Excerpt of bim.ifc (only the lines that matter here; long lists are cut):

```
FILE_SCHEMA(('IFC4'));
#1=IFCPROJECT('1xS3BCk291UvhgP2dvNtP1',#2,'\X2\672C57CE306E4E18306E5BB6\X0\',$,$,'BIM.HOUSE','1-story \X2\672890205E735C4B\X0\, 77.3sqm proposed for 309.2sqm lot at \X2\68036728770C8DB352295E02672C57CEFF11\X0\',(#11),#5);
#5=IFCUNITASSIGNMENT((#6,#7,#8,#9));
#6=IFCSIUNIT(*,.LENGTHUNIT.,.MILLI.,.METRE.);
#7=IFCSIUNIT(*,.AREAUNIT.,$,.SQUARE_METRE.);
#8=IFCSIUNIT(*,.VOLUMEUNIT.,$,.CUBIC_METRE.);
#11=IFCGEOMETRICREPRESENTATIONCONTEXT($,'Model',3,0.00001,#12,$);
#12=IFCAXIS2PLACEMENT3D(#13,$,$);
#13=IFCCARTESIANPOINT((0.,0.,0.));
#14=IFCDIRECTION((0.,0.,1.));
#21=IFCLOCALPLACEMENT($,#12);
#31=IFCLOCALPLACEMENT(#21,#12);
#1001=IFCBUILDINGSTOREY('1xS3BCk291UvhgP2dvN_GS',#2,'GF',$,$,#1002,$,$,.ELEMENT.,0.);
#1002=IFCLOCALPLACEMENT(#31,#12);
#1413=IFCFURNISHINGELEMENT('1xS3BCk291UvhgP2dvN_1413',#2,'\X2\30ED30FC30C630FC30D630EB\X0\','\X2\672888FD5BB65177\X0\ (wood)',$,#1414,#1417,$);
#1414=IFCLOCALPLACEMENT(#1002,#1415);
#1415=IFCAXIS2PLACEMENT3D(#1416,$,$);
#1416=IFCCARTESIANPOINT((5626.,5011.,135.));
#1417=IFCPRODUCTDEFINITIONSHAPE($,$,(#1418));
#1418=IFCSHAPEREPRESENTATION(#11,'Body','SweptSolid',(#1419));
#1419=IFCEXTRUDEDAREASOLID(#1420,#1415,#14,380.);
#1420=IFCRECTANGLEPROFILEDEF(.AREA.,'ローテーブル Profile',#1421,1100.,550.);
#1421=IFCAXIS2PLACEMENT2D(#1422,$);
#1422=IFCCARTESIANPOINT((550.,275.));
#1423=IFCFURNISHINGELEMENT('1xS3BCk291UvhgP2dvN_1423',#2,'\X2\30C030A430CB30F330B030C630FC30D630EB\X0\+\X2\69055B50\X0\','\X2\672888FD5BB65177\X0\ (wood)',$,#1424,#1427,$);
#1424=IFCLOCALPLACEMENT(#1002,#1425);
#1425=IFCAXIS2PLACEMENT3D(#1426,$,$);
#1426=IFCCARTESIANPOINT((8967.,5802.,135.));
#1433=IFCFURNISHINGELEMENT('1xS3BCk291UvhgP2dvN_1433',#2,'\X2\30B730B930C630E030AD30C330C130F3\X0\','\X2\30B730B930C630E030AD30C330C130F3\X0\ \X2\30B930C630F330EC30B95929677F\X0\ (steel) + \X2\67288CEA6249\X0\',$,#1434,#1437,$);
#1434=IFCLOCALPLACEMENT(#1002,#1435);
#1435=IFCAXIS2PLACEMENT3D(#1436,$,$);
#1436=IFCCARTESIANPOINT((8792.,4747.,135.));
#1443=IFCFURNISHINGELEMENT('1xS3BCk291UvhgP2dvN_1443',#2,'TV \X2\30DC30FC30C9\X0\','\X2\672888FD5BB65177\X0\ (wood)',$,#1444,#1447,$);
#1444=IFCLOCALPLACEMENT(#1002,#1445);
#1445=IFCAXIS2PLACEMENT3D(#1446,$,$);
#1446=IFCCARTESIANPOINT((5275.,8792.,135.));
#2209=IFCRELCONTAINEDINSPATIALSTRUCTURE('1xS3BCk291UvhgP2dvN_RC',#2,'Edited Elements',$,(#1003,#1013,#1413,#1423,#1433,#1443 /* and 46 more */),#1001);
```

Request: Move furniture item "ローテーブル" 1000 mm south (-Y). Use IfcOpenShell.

```python
import ifcopenshell
import ifcopenshell.api.geometry
import ifcopenshell.util.placement

model = ifcopenshell.open("bim.ifc")

item = model.by_id(1413)
matrix = ifcopenshell.util.placement.get_local_placement(item.ObjectPlacement)
matrix[1, 3] -= 1000.0
ifcopenshell.api.geometry.edit_object_placement(model, product=item, matrix=matrix, is_si=False)

print(ifcopenshell.util.placement.get_local_placement(item.ObjectPlacement).round(3) + 0.0)

model.write("bim_v2.ifc")
```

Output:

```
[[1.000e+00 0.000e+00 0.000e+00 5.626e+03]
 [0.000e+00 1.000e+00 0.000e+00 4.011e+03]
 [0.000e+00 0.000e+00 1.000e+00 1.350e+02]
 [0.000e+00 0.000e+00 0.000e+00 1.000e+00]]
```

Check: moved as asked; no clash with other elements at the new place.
